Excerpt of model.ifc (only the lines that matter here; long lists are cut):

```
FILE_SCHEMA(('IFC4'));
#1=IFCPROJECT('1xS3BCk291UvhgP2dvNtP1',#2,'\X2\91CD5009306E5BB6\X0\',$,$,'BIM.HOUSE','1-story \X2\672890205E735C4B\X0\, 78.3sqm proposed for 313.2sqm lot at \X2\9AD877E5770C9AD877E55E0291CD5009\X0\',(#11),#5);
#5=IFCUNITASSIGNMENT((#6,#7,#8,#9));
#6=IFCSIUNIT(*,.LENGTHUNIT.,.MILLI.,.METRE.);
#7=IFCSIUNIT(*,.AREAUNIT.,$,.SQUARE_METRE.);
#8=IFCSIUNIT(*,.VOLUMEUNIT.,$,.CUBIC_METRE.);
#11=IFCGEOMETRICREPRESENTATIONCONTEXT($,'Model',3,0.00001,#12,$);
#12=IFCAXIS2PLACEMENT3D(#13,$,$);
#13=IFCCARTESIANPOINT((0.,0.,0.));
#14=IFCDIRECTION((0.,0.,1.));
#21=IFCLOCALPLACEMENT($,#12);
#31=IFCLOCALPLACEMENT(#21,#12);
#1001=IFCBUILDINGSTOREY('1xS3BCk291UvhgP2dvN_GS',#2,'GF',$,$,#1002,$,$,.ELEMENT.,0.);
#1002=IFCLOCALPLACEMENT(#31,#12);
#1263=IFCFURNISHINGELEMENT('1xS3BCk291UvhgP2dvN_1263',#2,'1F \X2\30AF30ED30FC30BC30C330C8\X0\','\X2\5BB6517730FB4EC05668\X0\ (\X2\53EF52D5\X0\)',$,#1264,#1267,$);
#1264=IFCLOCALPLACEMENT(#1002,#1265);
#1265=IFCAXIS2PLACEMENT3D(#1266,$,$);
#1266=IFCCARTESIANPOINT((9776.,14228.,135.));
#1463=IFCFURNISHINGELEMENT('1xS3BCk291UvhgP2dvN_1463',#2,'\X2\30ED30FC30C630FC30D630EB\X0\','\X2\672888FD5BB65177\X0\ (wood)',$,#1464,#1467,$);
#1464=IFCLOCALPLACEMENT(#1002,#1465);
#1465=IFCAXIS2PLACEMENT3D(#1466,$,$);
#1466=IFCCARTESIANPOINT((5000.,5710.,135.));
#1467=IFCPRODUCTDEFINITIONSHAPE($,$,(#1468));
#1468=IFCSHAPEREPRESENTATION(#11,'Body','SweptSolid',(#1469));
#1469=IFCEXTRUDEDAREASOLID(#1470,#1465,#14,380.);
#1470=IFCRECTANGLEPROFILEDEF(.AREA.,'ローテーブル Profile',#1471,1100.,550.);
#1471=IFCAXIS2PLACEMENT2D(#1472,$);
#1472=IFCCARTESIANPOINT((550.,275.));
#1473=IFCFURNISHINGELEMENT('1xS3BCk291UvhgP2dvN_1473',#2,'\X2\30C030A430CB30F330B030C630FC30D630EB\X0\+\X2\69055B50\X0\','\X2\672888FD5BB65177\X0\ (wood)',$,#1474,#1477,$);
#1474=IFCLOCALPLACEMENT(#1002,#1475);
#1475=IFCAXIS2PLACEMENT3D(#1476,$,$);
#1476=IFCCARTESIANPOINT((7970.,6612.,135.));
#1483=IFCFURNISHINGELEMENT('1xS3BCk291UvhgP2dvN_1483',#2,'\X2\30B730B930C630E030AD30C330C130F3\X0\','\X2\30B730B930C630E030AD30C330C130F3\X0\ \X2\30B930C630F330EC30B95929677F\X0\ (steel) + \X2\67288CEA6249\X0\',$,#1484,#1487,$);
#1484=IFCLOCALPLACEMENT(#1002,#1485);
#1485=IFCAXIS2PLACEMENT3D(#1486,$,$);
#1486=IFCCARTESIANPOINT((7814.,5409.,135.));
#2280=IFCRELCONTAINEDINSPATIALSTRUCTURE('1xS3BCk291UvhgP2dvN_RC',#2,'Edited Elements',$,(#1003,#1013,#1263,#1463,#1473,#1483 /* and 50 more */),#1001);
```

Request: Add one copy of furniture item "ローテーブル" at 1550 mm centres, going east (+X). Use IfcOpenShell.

```python
import numpy as np
import ifcopenshell
import ifcopenshell.api.geometry
import ifcopenshell.api.root
import ifcopenshell.util.element
import ifcopenshell.util.placement
import ifcopenshell.util.unit

model = ifcopenshell.open("model.ifc")
unit_scale = ifcopenshell.util.unit.calculate_unit_scale(model)


def reuse_history(source, copy):
    """copy_class also copies each property set's owner history, people and application; keep the originals."""
    for rel in copy.IsDefinedBy:
        if rel.is_a("IfcRelDefinesByProperties") and (history := rel.RelatingPropertyDefinition.OwnerHistory):
            rel.RelatingPropertyDefinition.OwnerHistory = source.OwnerHistory
            ifcopenshell.util.element.remove_deep2(model, history)


source = model.by_guid("1xS3BCk291UvhgP2dvN_1463")
base = ifcopenshell.util.placement.get_local_placement(source.ObjectPlacement)
step = np.array([1.0, 0.0, 0.0]) * 1.55 / unit_scale

for i in range(1, 2):
    copy = ifcopenshell.api.root.copy_class(model, product=source)
    copy.Representation = ifcopenshell.util.element.copy_deep(
        model, source.Representation, exclude=["IfcGeometricRepresentationContext", "IfcRepresentationMap"]
    )
    reuse_history(source, copy)
    matrix = base.copy()
    matrix[:3, 3] += i * step
    print("added at", matrix[:3, 3].round(3) + 0.0)
    ifcopenshell.api.geometry.edit_object_placement(model, product=copy, matrix=matrix, is_si=False)

model.write("model_rev.ifc")
```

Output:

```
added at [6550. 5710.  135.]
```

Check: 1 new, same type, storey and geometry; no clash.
